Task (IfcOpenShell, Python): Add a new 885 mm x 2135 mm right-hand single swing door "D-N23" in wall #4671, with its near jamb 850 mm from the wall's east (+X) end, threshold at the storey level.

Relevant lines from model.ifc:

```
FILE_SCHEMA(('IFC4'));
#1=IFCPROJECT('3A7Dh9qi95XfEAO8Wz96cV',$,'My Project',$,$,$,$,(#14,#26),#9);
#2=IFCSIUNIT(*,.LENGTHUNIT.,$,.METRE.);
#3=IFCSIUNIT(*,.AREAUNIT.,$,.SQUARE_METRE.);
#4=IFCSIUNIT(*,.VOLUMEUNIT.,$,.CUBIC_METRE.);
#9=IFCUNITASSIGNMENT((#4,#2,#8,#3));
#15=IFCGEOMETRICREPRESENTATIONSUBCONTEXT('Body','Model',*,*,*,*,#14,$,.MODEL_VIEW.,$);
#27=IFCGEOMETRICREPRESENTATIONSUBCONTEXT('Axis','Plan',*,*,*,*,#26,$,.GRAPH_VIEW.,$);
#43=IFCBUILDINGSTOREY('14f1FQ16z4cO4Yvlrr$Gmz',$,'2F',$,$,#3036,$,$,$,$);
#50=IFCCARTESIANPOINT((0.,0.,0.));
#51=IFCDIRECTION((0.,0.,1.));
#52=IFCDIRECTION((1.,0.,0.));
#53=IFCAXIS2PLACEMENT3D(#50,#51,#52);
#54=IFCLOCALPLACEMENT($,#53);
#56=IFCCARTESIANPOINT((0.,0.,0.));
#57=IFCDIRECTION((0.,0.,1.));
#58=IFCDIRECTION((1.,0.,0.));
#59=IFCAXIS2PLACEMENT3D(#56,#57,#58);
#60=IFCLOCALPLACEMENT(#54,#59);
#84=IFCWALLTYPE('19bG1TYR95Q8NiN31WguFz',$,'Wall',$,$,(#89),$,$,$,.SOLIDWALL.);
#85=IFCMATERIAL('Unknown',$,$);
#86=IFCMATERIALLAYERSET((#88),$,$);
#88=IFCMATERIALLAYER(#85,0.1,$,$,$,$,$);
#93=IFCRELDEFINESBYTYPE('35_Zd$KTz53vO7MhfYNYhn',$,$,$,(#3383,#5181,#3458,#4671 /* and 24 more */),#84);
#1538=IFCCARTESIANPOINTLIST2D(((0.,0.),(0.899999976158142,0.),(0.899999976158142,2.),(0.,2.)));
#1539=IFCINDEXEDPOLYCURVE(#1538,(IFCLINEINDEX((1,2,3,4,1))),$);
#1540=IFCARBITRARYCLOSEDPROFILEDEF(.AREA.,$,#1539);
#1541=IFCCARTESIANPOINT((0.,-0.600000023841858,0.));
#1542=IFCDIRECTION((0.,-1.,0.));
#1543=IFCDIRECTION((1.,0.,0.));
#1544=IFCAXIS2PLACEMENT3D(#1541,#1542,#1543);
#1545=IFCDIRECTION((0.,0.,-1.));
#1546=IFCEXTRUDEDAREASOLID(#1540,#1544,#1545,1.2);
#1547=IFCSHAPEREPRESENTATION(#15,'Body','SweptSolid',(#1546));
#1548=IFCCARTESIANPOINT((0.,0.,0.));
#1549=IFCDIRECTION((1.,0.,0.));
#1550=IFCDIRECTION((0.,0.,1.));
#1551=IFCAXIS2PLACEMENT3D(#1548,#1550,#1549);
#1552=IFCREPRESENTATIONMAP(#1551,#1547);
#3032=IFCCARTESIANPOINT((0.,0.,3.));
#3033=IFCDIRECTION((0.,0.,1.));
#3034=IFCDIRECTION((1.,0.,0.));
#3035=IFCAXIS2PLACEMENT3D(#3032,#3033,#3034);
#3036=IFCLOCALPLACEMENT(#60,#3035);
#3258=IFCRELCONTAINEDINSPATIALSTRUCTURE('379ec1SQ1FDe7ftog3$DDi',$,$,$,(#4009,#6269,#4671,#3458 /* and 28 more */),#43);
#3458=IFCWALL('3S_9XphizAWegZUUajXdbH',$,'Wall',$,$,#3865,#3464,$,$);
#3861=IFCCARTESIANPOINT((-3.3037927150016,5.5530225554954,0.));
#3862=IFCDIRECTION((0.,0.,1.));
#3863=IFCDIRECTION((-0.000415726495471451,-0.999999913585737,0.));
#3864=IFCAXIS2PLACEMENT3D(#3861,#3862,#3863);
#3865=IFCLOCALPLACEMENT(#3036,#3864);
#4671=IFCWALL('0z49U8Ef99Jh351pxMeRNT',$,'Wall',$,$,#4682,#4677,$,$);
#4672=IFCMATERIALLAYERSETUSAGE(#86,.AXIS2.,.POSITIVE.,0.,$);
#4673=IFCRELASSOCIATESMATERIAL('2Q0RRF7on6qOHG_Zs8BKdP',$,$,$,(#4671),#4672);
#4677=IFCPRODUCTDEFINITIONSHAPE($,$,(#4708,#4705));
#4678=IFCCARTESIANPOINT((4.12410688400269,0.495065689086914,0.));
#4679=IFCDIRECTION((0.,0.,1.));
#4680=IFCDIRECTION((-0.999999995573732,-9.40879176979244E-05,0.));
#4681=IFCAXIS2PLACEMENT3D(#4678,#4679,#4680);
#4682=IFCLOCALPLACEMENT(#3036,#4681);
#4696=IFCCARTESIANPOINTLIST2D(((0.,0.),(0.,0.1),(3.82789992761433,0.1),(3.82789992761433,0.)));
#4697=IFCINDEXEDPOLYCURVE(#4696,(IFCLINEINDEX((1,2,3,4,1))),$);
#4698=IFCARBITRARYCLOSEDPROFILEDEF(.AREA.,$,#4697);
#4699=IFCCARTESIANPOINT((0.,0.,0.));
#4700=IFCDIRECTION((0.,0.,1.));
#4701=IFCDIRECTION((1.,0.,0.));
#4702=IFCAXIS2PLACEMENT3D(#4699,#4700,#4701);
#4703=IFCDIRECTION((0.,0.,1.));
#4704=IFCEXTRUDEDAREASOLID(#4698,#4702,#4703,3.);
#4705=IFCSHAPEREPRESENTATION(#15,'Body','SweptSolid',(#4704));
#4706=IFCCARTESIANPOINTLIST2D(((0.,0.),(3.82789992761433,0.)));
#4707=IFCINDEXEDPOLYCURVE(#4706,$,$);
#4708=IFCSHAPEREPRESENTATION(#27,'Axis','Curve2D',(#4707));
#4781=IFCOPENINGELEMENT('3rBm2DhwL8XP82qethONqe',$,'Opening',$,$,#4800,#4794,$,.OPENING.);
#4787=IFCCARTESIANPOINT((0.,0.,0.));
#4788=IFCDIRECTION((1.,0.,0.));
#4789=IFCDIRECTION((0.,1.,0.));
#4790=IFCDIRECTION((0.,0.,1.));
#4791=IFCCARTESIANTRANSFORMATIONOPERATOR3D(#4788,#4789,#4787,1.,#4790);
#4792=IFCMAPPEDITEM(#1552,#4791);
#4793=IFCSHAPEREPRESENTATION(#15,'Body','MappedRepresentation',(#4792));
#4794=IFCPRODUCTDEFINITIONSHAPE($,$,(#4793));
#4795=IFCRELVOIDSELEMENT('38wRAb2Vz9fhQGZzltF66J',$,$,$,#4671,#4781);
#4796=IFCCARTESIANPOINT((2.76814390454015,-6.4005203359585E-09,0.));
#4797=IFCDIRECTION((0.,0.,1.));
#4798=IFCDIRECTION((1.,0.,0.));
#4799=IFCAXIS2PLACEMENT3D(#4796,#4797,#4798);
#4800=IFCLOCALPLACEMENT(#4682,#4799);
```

```python
import numpy as np
import ifcopenshell
import ifcopenshell.api.feature
import ifcopenshell.api.geometry
import ifcopenshell.api.root
import ifcopenshell.api.spatial
import ifcopenshell.geom
import ifcopenshell.util.element
import ifcopenshell.util.placement
import ifcopenshell.util.representation
import ifcopenshell.util.shape
import ifcopenshell.util.unit

model = ifcopenshell.open("model.ifc")
unit_scale = ifcopenshell.util.unit.calculate_unit_scale(model)
settings = ifcopenshell.geom.settings()


def volume(element):
    """Net volume in cubic metres, openings subtracted."""
    shape = ifcopenshell.geom.create_shape(settings, element)
    return ifcopenshell.util.shape.get_volume(shape.geometry)


wall = model.by_guid("0z49U8Ef99Jh351pxMeRNT")
storey = ifcopenshell.util.element.get_container(wall, ifc_class="IfcBuildingStorey")
context = ifcopenshell.util.representation.get_context(model, "Model", "Body", "MODEL_VIEW")
before = volume(wall)

width, height, from_end, sill = 0.885, 2.135, 0.85, 0.0  # metres

# The wall runs along its own X axis, and the end named is its -X end.
wall_shape = ifcopenshell.geom.create_shape(settings, wall)
x, y, z = ifcopenshell.util.shape.get_vertices(wall_shape.geometry).T
start = x.min() + from_end
face, thickness = float(y.min()), float(y.max() - y.min())
wall_matrix = ifcopenshell.util.placement.get_local_placement(wall.ObjectPlacement)
level = ifcopenshell.util.placement.get_local_placement(storey.ObjectPlacement)[2, 3]


def in_wall(x, y):
    """Placement at x, y metres in the wall's axes, at sill height."""
    matrix = wall_matrix.copy()
    matrix[:, 3] = wall_matrix @ np.array([x / unit_scale, y / unit_scale, 0.0, 1.0])
    matrix[2, 3] = level + sill / unit_scale
    return matrix


# Opening: a box that overshoots both wall faces by 50 mm.
opening = ifcopenshell.api.root.create_entity(model, ifc_class="IfcOpeningElement", predefined_type="OPENING")
box = ifcopenshell.api.geometry.add_wall_representation(
    model, context=context, length=width, height=height, thickness=thickness + 0.1
)
ifcopenshell.api.geometry.assign_representation(model, product=opening, representation=box)
ifcopenshell.api.geometry.edit_object_placement(model, product=opening, matrix=in_wall(start, face - 0.05), is_si=False)
ifcopenshell.api.feature.add_feature(model, feature=opening, element=wall)

door = ifcopenshell.api.root.create_entity(model, ifc_class="IfcDoor", name="D-N23", predefined_type="DOOR")
door.OverallWidth, door.OverallHeight = width / unit_scale, height / unit_scale
door.OperationType = "SINGLE_SWING_RIGHT"
body = ifcopenshell.api.geometry.add_door_representation(
    model,
    context=context,
    overall_width=door.OverallWidth,
    overall_height=door.OverallHeight,
    operation_type="SINGLE_SWING_RIGHT",
    lining_properties={"LiningDepth": thickness / unit_scale, "ThresholdDepth": thickness / unit_scale},
)
ifcopenshell.api.geometry.assign_representation(model, product=door, representation=body)
ifcopenshell.api.spatial.assign_container(model, products=[door], relating_structure=storey)
ifcopenshell.api.feature.add_filling(model, opening=opening, element=door)

# The lining spans the wall, so the door starts at the wall face.
ifcopenshell.api.geometry.edit_object_placement(model, product=door, matrix=in_wall(start, face), is_si=False)

after = volume(wall)

print(f"wall volume {before:.3f} -> {after:.3f} m3")

model.write("model_v2.ifc")
```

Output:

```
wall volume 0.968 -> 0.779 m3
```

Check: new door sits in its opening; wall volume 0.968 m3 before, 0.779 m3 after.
